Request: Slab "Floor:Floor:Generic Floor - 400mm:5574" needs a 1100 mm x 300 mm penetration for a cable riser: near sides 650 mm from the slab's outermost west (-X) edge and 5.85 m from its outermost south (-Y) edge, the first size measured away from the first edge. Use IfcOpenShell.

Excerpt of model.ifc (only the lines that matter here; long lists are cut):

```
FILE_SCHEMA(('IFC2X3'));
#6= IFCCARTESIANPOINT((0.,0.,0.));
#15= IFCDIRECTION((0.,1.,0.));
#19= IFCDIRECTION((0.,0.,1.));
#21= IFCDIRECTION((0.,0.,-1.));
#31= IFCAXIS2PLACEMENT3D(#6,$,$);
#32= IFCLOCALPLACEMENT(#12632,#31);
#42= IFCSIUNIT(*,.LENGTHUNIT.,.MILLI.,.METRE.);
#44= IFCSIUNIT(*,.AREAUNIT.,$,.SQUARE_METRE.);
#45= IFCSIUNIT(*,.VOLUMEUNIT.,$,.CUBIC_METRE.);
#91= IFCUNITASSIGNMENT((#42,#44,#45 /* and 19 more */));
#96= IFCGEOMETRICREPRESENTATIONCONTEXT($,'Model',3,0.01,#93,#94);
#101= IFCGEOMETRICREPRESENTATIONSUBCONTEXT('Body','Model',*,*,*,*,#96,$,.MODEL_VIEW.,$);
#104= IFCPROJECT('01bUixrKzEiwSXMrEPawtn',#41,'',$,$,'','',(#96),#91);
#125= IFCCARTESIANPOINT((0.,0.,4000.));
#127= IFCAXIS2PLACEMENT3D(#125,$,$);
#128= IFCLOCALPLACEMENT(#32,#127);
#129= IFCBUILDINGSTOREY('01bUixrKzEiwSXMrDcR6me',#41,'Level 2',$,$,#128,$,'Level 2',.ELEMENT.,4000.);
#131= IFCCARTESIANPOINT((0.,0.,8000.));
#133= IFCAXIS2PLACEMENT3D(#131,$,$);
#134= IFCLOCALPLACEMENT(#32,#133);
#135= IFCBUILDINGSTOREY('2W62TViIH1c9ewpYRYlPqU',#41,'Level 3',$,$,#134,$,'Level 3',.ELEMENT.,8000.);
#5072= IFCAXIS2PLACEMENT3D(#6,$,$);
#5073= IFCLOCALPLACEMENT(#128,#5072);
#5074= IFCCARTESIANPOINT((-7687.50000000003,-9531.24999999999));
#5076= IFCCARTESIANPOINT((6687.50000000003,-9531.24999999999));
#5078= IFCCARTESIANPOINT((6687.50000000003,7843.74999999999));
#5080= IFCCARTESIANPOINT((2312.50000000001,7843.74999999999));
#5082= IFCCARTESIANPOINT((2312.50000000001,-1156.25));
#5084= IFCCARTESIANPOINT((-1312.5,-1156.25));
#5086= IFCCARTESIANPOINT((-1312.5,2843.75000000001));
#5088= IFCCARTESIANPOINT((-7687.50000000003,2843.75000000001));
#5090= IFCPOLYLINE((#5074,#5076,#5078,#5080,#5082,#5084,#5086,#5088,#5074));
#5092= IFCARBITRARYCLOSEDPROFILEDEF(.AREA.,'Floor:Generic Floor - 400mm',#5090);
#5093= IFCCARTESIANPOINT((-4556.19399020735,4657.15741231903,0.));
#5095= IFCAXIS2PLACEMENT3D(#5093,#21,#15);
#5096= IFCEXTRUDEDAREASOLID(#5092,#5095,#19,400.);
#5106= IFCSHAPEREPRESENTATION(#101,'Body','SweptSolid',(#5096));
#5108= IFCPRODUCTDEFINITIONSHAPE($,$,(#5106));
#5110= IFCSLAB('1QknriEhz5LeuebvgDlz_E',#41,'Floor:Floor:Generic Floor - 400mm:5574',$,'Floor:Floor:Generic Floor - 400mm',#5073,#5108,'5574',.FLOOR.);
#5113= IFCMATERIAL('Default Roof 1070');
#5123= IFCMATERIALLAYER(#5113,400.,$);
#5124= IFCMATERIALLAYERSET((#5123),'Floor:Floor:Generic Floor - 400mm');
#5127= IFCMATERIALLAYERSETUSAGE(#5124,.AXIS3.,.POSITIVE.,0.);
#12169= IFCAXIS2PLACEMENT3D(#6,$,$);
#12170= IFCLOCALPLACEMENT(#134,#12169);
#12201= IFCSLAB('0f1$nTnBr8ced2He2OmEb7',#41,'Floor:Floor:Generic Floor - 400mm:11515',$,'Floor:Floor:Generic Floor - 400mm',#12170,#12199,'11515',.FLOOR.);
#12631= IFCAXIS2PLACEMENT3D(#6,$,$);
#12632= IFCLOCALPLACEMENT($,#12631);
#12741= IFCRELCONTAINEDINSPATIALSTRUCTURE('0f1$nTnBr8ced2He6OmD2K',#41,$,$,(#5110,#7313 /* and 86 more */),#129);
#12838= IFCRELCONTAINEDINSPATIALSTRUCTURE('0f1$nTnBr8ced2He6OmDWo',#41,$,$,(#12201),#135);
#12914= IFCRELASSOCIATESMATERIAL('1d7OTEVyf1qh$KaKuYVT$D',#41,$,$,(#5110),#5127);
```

```python
import numpy as np
import ifcopenshell
import ifcopenshell.api.feature
import ifcopenshell.api.geometry
import ifcopenshell.api.root
import ifcopenshell.geom
import ifcopenshell.util.placement
import ifcopenshell.util.representation
import ifcopenshell.util.shape
import ifcopenshell.util.unit

model = ifcopenshell.open("model.ifc")
unit_scale = ifcopenshell.util.unit.calculate_unit_scale(model)
settings = ifcopenshell.geom.settings()


def volume(element):
    """Net volume in cubic metres, openings subtracted."""
    shape = ifcopenshell.geom.create_shape(settings, element)
    return ifcopenshell.util.shape.get_volume(shape.geometry)


slab = model.by_guid("1QknriEhz5LeuebvgDlz_E")
before = volume(slab)

# Extent in the slab's own axes, in metres. The edges named are its -X and -Y sides.
slab_shape = ifcopenshell.geom.create_shape(settings, slab)
vertices = ifcopenshell.util.shape.get_vertices(slab_shape.geometry)
x_min, y_min, bottom = vertices.min(axis=0)
top = vertices[:, 2].max()

opening = ifcopenshell.api.root.create_entity(model, ifc_class="IfcOpeningElement", name="Cable riser opening")
context = ifcopenshell.util.representation.get_context(model, "Model", "Body", "MODEL_VIEW")
width, depth = 1.1, 0.3
outline = [(0.0, 0.0), (width, 0.0), (width, depth), (0.0, depth), (0.0, 0.0)]
# Overshoot both faces by 50 mm so the cut is clean.
shape = ifcopenshell.api.geometry.add_slab_representation(
    model, context=context, depth=top - bottom + 0.1, polyline=outline
)
ifcopenshell.api.geometry.assign_representation(model, product=opening, representation=shape)

matrix = ifcopenshell.util.placement.get_local_placement(slab.ObjectPlacement)
matrix[:, 3] = matrix @ np.append(np.array([x_min + 0.65, y_min + 5.85, bottom - 0.05]) / unit_scale, 1.0)
ifcopenshell.api.geometry.edit_object_placement(model, product=opening, matrix=matrix, is_si=False)
ifcopenshell.api.feature.add_feature(model, feature=opening, element=slab)

after = volume(slab)

print(f"slab volume {before:.3f} -> {after:.3f} m3")

model.write("model-out.ifc")
```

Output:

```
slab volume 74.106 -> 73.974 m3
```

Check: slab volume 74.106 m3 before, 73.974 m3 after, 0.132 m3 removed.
